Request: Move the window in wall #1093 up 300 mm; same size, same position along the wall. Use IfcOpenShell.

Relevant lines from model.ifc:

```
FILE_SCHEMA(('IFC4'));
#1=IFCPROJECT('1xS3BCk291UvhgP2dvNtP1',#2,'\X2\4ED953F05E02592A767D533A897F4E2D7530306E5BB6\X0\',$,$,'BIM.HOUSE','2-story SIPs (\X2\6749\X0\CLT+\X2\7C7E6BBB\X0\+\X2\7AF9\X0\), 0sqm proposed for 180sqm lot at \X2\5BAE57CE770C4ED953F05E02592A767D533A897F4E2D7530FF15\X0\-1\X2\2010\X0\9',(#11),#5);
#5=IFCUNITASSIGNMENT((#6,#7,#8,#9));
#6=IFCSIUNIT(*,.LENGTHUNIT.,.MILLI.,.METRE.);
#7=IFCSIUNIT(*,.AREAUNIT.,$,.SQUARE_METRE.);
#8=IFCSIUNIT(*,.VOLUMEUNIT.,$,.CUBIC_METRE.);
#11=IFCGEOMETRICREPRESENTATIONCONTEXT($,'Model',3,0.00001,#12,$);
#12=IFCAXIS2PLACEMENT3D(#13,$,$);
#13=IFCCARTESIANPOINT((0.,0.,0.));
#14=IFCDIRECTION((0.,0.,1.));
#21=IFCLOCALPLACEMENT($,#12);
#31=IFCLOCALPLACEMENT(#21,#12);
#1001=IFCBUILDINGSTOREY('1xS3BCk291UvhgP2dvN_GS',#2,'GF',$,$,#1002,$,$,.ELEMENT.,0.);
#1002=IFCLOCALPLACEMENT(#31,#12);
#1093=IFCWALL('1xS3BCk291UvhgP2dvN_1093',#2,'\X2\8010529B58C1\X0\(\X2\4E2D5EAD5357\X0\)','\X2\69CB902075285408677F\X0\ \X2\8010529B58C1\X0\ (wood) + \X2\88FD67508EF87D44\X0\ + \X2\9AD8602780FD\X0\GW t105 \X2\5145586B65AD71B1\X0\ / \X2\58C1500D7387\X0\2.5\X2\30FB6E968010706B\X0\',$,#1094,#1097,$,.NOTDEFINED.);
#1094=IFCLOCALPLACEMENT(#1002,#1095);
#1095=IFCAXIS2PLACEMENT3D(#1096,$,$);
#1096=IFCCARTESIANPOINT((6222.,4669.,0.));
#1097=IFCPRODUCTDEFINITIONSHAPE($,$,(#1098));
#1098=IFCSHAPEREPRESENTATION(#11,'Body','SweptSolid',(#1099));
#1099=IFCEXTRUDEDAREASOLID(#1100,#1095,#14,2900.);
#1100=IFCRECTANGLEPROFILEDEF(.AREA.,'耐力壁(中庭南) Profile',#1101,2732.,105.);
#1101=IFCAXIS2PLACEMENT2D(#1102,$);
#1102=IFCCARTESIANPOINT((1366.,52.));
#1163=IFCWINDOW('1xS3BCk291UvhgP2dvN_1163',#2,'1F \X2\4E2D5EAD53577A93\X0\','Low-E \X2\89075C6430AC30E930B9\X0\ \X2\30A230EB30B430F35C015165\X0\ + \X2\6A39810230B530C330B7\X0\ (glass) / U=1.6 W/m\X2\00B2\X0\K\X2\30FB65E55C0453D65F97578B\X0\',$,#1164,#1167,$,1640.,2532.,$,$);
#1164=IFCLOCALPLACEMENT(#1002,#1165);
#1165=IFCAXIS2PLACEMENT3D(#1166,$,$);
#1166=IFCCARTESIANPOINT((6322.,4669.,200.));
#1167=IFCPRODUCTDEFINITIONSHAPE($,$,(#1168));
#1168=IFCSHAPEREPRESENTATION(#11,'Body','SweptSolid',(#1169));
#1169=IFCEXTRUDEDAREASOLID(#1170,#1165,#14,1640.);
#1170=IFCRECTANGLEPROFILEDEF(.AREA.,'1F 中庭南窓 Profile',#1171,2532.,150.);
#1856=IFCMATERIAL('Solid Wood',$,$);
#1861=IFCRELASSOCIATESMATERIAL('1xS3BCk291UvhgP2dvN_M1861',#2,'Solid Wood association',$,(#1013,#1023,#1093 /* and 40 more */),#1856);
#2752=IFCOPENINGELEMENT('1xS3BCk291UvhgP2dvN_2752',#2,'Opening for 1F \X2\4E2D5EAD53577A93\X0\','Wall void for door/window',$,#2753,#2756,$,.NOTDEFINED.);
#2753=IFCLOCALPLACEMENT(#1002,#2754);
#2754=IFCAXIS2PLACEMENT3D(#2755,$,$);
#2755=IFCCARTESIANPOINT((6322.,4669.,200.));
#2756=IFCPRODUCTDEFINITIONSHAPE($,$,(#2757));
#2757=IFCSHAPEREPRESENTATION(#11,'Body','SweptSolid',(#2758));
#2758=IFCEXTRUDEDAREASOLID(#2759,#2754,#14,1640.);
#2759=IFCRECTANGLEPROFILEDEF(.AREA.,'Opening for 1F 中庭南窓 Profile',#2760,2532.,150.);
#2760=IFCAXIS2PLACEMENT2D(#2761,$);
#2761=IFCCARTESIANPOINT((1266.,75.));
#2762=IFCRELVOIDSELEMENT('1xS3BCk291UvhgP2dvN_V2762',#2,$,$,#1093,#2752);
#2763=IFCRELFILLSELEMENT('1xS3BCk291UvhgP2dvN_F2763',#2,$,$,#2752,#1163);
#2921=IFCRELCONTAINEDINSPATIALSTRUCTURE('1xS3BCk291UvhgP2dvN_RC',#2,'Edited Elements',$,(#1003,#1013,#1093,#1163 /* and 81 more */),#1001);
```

```python
import numpy as np
import ifcopenshell
import ifcopenshell.api.geometry
import ifcopenshell.util.placement
import ifcopenshell.util.unit

model = ifcopenshell.open("model.ifc")
unit_scale = ifcopenshell.util.unit.calculate_unit_scale(model)

window = model.by_id(1163)
opening = window.FillsVoids[0].RelatingOpeningElement
dz = 0.3 / unit_scale

shift = np.array([0.0, 0.0, dz])
# The window is not placed relative to its opening, so move both.
for product in (opening, window):
    matrix = ifcopenshell.util.placement.get_local_placement(product.ObjectPlacement)
    matrix[:3, 3] += shift
    ifcopenshell.api.geometry.edit_object_placement(model, product=product, matrix=matrix, is_si=False)

print(f"moved by {dz * unit_scale:+.3f} m")

model.write("model-out.ifc")
```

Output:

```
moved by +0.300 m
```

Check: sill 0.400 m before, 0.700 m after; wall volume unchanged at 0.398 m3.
